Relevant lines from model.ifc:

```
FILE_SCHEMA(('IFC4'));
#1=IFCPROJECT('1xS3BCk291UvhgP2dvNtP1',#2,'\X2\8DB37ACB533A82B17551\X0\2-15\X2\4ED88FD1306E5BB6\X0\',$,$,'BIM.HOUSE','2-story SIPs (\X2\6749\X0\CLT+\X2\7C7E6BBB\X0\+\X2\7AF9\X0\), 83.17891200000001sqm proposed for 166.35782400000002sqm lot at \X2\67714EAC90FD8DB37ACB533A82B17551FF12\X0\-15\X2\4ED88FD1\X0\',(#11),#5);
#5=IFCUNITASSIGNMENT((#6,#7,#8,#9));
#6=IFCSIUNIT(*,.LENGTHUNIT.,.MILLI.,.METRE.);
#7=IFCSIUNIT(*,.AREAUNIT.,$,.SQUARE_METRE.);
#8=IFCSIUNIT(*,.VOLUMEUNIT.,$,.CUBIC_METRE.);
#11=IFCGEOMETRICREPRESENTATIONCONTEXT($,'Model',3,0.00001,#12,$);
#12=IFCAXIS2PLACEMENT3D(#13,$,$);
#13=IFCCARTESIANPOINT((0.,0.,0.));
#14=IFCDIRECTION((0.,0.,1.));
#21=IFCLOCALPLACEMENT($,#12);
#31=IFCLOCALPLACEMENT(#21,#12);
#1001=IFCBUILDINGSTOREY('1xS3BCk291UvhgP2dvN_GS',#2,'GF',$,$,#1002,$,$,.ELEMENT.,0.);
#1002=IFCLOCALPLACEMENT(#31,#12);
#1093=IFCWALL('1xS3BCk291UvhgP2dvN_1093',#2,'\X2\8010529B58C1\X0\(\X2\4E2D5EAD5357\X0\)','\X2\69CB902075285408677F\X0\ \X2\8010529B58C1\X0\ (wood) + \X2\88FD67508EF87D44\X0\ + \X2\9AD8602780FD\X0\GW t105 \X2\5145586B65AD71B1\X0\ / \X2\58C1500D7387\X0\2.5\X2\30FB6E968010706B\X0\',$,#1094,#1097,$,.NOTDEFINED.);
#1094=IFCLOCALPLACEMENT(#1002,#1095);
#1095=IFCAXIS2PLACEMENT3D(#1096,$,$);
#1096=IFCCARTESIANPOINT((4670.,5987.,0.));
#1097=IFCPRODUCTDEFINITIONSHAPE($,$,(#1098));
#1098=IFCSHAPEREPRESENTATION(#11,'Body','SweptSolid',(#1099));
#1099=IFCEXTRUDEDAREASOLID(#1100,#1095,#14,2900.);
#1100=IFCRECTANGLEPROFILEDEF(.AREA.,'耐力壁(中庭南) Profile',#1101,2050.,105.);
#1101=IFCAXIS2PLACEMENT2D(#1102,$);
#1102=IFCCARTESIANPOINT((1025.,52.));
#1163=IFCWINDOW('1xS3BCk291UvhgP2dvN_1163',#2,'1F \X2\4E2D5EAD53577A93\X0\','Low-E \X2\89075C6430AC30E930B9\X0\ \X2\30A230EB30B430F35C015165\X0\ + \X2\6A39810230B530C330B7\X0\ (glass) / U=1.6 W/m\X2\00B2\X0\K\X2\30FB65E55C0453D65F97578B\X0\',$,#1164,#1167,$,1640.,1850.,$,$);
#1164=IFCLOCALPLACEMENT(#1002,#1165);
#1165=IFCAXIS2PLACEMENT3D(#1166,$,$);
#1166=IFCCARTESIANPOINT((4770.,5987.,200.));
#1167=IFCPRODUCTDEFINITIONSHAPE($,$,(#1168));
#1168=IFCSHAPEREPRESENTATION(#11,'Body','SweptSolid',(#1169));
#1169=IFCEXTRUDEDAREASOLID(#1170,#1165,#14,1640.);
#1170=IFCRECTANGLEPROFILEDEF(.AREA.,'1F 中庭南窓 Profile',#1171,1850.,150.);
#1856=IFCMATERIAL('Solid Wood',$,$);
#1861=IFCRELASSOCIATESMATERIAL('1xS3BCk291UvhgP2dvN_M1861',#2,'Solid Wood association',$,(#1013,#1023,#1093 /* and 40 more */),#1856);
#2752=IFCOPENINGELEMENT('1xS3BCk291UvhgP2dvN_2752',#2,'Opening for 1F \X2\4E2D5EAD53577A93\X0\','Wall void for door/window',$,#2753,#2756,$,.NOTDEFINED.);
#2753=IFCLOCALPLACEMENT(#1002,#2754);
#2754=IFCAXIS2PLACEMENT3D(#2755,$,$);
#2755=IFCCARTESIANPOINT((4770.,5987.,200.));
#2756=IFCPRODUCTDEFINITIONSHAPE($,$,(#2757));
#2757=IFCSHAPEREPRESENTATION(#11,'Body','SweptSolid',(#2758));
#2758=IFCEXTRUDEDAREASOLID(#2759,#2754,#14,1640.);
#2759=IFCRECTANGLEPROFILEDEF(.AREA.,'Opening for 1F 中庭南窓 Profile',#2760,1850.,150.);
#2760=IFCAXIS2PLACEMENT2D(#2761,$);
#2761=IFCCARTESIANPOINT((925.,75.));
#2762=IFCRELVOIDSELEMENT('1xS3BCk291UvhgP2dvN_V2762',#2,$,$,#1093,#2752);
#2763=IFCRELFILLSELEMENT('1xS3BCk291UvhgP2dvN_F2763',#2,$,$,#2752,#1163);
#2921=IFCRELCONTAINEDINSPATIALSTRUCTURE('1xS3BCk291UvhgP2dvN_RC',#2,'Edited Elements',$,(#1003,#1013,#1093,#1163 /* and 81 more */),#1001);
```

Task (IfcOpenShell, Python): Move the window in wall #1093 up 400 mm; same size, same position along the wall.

```python
import numpy as np
import ifcopenshell
import ifcopenshell.api.geometry
import ifcopenshell.util.placement
import ifcopenshell.util.unit

model = ifcopenshell.open("model.ifc")
unit_scale = ifcopenshell.util.unit.calculate_unit_scale(model)

window = model.by_guid("1xS3BCk291UvhgP2dvN_1163")
opening = window.FillsVoids[0].RelatingOpeningElement
dz = 400.0

shift = np.array([0.0, 0.0, dz])
# The window is not placed relative to its opening, so move both.
for product in (opening, window):
    matrix = ifcopenshell.util.placement.get_local_placement(product.ObjectPlacement)
    matrix[:3, 3] += shift
    ifcopenshell.api.geometry.edit_object_placement(model, product=product, matrix=matrix, is_si=False)

print(f"moved by {dz * unit_scale:+.3f} m")

model.write("model_v2.ifc")
```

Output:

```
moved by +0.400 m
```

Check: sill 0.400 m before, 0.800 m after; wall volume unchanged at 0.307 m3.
